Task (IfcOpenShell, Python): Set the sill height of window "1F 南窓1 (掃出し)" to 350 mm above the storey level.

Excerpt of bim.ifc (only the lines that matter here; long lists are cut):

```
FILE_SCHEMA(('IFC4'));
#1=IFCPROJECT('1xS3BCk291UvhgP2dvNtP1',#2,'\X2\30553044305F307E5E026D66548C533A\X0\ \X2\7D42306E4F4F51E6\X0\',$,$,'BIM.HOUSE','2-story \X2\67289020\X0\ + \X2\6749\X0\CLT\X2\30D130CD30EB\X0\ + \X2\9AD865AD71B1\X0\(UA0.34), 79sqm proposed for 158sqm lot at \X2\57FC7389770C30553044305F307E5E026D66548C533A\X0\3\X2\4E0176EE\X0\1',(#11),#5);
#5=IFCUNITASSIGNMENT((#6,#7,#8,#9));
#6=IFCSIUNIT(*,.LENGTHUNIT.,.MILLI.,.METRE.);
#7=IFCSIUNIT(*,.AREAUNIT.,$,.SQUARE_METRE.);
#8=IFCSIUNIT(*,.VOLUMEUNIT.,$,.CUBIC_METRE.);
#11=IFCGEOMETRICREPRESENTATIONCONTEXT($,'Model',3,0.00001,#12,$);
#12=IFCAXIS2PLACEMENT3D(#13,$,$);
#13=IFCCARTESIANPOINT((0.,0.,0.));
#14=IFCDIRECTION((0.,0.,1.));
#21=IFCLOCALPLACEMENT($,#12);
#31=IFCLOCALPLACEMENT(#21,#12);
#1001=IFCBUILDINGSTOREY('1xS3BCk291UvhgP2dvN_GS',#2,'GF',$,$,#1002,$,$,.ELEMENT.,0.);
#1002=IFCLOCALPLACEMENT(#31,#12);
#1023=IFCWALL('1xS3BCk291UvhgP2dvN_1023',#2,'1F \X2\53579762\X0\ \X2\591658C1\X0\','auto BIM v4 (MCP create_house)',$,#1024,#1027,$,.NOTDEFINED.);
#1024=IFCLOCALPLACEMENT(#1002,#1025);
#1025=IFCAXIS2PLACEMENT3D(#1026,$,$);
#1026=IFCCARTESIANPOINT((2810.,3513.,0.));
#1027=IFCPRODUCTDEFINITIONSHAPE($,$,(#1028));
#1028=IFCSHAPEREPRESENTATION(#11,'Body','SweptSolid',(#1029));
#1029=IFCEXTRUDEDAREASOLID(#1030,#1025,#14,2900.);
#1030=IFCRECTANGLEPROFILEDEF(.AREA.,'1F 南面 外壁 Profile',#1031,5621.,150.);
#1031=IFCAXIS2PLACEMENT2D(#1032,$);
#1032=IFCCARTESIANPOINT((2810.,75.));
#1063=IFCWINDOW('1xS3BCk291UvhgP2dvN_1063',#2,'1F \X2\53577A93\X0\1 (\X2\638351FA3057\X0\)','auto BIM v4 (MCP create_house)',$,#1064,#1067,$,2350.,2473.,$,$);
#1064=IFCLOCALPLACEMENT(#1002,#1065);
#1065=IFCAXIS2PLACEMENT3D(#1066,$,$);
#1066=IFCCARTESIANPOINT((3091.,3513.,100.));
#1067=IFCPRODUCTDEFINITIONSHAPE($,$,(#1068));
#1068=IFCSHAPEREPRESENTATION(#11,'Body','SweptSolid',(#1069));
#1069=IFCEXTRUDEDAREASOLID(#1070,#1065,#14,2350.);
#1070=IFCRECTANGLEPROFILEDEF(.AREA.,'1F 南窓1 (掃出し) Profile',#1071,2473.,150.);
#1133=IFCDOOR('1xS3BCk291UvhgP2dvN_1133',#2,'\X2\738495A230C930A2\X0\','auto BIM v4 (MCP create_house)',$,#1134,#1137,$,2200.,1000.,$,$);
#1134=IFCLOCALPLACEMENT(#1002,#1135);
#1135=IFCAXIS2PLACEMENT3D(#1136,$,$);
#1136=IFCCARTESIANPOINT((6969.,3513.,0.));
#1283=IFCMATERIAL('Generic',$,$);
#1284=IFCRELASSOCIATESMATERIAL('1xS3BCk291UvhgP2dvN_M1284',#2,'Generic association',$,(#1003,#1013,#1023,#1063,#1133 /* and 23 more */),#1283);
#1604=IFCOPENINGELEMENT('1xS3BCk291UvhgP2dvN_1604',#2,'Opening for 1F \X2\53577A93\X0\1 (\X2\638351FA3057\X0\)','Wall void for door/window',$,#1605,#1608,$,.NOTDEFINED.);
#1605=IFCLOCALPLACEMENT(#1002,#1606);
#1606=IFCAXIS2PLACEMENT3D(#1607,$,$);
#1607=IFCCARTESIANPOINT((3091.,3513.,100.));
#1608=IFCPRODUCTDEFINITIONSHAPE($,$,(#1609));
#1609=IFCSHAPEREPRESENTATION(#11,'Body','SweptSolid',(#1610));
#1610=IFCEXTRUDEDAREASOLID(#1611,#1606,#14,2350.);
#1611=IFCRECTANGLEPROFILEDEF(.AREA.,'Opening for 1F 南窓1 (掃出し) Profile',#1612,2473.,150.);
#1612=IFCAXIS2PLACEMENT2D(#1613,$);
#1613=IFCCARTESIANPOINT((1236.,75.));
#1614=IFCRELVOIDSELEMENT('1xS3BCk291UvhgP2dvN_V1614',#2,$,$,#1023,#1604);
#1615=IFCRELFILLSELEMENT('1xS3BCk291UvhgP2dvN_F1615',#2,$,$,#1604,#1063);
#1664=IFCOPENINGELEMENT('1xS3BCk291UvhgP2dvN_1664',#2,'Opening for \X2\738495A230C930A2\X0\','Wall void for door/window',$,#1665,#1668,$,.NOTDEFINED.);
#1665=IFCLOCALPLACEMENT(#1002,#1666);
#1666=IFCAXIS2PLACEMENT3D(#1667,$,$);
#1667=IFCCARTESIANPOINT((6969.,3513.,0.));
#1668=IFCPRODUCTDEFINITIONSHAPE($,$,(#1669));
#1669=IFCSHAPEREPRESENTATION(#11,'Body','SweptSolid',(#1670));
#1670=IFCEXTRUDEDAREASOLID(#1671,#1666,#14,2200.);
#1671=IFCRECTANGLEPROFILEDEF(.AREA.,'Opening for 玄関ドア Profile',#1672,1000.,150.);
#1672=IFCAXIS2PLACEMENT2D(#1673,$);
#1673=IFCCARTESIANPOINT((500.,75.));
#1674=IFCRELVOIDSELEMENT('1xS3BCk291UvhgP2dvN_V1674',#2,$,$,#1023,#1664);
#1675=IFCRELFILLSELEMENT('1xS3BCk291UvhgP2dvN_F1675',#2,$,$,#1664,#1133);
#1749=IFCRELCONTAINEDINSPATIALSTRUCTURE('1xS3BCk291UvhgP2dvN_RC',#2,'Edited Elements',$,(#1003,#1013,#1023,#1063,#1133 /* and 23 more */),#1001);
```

```python
import numpy as np
import ifcopenshell
import ifcopenshell.api.geometry
import ifcopenshell.geom
import ifcopenshell.util.element
import ifcopenshell.util.placement
import ifcopenshell.util.shape
import ifcopenshell.util.unit

model = ifcopenshell.open("bim.ifc")
unit_scale = ifcopenshell.util.unit.calculate_unit_scale(model)

window = model.by_guid("1xS3BCk291UvhgP2dvN_1063")
opening = window.FillsVoids[0].RelatingOpeningElement
storey = ifcopenshell.util.element.get_container(window, ifc_class="IfcBuildingStorey")
level = ifcopenshell.util.placement.get_local_placement(storey.ObjectPlacement)[2, 3]

# The opening's origin need not be at the sill, so measure its lowest point.
shape = ifcopenshell.geom.create_shape(ifcopenshell.geom.settings(), opening)
bottom = ifcopenshell.util.shape.get_shape_bottom_elevation(shape, shape.geometry) / unit_scale
dz = level + 350.0 - bottom

shift = np.array([0.0, 0.0, dz])
# The window is not placed relative to its opening, so move both.
for product in (opening, window):
    matrix = ifcopenshell.util.placement.get_local_placement(product.ObjectPlacement)
    matrix[:3, 3] += shift
    ifcopenshell.api.geometry.edit_object_placement(model, product=product, matrix=matrix, is_si=False)

print(f"moved by {dz * unit_scale:+.3f} m")

model.write("bim_rev.ifc")
```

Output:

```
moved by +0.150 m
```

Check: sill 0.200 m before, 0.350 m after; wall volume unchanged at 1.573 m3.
